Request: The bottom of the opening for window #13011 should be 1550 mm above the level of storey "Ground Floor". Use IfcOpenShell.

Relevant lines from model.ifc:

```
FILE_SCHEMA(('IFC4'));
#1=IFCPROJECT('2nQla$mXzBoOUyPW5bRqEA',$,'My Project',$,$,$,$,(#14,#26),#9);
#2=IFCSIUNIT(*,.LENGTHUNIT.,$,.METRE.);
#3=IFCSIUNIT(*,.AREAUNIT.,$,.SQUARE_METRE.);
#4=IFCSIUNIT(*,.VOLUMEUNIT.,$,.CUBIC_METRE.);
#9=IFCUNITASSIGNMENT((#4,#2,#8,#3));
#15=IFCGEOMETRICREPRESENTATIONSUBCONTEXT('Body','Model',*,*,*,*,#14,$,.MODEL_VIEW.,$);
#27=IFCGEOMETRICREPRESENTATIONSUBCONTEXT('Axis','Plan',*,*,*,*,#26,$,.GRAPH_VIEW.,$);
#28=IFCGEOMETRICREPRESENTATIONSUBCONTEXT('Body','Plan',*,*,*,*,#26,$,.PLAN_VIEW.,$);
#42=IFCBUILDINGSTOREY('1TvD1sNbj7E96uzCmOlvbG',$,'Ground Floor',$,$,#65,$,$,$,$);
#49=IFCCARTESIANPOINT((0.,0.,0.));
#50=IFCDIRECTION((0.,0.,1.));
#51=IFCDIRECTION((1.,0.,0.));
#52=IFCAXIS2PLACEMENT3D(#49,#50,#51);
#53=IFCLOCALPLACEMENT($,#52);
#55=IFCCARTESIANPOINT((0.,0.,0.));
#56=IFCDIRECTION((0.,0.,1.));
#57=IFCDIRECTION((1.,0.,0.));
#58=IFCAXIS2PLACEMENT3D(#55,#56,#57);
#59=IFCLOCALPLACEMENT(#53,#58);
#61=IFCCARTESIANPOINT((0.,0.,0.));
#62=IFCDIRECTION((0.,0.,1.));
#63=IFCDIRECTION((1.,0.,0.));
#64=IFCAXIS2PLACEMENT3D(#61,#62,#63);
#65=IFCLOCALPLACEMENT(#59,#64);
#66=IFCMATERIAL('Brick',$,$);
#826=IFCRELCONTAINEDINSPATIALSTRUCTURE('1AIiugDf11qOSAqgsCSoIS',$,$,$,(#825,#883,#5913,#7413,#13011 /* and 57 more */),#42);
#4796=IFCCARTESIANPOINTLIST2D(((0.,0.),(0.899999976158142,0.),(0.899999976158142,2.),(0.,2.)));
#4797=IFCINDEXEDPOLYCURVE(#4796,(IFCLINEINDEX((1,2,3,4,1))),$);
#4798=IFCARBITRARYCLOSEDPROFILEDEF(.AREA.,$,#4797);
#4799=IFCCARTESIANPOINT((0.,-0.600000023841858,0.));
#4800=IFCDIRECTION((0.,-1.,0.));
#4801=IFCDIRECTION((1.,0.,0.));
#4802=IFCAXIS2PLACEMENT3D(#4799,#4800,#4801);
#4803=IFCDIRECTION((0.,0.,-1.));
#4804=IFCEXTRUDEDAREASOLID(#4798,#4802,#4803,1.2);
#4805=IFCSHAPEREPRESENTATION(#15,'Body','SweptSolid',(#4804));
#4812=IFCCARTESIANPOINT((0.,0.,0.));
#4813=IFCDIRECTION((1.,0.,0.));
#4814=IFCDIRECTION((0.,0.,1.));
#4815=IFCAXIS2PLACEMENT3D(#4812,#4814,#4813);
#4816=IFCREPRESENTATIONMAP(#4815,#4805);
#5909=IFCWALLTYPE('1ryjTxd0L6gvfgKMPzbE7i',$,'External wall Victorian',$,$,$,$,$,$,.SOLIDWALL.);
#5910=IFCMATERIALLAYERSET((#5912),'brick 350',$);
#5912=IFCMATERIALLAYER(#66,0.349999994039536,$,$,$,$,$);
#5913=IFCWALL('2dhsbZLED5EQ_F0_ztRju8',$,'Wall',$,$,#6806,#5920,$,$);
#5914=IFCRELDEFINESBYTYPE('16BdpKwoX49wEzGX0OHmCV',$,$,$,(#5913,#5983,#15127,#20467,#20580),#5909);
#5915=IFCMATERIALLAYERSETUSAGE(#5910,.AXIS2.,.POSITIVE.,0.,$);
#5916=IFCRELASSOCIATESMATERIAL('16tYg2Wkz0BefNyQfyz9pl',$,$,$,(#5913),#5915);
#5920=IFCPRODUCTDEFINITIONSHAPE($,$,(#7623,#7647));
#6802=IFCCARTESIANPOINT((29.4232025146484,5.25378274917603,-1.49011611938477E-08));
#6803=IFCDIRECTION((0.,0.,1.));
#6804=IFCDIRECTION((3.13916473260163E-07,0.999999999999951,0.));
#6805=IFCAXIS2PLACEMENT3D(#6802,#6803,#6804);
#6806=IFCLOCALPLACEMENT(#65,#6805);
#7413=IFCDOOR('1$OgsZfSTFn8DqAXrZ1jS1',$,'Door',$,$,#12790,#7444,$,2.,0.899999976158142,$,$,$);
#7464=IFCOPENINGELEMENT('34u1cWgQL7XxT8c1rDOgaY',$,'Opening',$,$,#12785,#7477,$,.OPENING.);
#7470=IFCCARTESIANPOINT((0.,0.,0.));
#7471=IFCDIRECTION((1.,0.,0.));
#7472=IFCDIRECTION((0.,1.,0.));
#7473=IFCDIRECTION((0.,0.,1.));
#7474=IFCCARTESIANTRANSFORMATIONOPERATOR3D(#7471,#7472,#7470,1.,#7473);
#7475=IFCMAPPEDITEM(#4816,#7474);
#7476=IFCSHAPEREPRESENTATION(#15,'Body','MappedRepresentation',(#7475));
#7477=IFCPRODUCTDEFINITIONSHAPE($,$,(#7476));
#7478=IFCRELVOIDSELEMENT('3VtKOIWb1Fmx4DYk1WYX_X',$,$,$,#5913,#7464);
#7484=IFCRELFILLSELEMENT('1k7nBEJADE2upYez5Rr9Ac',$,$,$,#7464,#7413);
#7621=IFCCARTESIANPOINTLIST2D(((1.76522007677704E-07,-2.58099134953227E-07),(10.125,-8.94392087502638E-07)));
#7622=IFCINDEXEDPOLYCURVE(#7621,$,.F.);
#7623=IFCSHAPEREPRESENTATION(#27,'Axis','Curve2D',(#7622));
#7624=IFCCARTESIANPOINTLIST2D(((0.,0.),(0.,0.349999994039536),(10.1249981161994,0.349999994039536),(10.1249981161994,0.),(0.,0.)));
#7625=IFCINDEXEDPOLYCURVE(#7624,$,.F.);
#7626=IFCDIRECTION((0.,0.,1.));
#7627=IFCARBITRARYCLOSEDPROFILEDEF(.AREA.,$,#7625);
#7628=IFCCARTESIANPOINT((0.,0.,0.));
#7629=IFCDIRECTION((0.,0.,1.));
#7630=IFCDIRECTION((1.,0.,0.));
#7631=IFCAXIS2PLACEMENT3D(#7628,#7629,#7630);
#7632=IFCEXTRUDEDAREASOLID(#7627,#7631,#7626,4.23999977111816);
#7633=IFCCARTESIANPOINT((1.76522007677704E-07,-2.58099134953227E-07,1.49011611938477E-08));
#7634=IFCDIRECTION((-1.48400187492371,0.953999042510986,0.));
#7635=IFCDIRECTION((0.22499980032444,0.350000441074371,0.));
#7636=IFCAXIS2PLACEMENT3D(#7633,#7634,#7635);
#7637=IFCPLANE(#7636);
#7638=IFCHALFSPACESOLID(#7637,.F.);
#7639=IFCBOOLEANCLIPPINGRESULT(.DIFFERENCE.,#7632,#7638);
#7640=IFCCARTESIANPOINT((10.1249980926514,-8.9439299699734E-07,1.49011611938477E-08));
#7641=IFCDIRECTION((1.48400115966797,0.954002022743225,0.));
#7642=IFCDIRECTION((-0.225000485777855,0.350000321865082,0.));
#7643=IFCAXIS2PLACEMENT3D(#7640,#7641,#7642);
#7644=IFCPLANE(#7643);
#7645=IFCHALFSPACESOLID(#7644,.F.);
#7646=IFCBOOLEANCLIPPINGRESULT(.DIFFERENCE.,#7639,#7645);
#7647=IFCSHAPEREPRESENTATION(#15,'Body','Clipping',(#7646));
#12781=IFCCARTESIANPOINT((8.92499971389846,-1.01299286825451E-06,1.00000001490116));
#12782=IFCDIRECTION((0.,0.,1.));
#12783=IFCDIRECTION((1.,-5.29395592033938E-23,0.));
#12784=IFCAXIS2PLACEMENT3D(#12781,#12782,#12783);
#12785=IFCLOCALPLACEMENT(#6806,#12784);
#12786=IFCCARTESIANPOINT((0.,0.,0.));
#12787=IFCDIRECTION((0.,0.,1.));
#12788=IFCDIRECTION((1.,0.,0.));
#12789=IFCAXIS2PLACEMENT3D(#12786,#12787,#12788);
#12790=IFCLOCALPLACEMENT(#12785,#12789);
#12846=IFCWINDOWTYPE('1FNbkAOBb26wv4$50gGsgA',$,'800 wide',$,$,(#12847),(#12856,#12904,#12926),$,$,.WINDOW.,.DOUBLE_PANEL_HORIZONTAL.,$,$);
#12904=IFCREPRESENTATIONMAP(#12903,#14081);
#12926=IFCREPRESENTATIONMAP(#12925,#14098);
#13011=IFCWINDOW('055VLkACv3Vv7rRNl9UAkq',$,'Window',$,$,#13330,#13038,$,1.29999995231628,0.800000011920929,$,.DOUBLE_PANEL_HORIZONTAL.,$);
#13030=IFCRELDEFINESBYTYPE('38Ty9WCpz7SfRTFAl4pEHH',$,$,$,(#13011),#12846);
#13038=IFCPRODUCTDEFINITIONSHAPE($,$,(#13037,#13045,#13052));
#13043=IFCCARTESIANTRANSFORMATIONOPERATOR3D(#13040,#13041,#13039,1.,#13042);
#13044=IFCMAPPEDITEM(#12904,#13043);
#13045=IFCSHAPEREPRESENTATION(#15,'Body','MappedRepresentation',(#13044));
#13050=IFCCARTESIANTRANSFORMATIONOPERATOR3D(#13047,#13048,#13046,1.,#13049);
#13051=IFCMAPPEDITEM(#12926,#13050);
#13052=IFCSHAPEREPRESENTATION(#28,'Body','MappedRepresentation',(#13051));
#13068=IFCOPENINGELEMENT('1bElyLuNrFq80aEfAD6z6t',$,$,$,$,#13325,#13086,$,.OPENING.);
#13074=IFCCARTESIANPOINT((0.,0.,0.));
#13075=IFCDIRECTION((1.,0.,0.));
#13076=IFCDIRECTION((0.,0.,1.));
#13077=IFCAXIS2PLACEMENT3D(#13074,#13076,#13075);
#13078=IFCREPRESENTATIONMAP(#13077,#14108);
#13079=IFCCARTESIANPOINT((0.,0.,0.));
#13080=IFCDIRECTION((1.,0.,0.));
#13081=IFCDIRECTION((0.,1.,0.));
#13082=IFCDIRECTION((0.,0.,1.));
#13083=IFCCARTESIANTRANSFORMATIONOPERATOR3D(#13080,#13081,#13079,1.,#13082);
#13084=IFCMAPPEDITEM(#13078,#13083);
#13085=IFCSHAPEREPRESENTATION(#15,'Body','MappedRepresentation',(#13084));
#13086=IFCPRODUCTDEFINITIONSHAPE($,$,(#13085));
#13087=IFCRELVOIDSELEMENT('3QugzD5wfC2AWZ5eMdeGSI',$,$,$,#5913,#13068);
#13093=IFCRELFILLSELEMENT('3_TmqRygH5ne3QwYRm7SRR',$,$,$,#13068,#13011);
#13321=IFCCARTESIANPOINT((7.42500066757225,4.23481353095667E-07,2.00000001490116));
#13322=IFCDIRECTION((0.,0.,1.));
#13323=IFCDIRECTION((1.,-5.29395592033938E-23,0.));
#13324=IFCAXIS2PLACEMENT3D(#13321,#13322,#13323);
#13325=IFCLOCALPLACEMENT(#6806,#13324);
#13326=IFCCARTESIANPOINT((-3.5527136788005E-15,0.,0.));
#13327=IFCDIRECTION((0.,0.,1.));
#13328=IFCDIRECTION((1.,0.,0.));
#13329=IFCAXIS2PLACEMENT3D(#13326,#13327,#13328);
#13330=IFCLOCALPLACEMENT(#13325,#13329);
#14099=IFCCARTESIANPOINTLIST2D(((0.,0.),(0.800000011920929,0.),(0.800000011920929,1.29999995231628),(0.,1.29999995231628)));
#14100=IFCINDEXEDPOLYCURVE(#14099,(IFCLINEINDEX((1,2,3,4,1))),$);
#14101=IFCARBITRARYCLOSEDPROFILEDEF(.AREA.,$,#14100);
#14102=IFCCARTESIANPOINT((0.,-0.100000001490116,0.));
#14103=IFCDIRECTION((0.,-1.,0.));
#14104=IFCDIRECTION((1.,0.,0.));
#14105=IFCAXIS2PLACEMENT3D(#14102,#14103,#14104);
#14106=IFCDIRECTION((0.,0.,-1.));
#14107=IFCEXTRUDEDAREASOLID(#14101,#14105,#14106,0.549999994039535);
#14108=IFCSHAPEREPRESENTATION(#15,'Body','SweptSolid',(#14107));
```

```python
import numpy as np
import ifcopenshell
import ifcopenshell.api.geometry
import ifcopenshell.geom
import ifcopenshell.util.element
import ifcopenshell.util.placement
import ifcopenshell.util.shape
import ifcopenshell.util.unit

model = ifcopenshell.open("model.ifc")
unit_scale = ifcopenshell.util.unit.calculate_unit_scale(model)

window = model.by_id(13011)
opening = window.FillsVoids[0].RelatingOpeningElement
storey = ifcopenshell.util.element.get_container(window, ifc_class="IfcBuildingStorey")
level = ifcopenshell.util.placement.get_local_placement(storey.ObjectPlacement)[2, 3]

# The opening's origin need not be at the sill, so measure its lowest point.
shape = ifcopenshell.geom.create_shape(ifcopenshell.geom.settings(), opening)
bottom = ifcopenshell.util.shape.get_shape_bottom_elevation(shape, shape.geometry) / unit_scale
dz = level + 1.55 - bottom

shift = np.array([0.0, 0.0, dz])
# The window is placed relative to its opening, so it follows when the opening moves.
matrix = ifcopenshell.util.placement.get_local_placement(opening.ObjectPlacement)
matrix[:3, 3] += shift
ifcopenshell.api.geometry.edit_object_placement(
    model, product=opening, matrix=matrix, is_si=False, should_transform_children=True
)

print(f"moved by {dz * unit_scale:+.3f} m")

model.write("model_updated.ifc")
```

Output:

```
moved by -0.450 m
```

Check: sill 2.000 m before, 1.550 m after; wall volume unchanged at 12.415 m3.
